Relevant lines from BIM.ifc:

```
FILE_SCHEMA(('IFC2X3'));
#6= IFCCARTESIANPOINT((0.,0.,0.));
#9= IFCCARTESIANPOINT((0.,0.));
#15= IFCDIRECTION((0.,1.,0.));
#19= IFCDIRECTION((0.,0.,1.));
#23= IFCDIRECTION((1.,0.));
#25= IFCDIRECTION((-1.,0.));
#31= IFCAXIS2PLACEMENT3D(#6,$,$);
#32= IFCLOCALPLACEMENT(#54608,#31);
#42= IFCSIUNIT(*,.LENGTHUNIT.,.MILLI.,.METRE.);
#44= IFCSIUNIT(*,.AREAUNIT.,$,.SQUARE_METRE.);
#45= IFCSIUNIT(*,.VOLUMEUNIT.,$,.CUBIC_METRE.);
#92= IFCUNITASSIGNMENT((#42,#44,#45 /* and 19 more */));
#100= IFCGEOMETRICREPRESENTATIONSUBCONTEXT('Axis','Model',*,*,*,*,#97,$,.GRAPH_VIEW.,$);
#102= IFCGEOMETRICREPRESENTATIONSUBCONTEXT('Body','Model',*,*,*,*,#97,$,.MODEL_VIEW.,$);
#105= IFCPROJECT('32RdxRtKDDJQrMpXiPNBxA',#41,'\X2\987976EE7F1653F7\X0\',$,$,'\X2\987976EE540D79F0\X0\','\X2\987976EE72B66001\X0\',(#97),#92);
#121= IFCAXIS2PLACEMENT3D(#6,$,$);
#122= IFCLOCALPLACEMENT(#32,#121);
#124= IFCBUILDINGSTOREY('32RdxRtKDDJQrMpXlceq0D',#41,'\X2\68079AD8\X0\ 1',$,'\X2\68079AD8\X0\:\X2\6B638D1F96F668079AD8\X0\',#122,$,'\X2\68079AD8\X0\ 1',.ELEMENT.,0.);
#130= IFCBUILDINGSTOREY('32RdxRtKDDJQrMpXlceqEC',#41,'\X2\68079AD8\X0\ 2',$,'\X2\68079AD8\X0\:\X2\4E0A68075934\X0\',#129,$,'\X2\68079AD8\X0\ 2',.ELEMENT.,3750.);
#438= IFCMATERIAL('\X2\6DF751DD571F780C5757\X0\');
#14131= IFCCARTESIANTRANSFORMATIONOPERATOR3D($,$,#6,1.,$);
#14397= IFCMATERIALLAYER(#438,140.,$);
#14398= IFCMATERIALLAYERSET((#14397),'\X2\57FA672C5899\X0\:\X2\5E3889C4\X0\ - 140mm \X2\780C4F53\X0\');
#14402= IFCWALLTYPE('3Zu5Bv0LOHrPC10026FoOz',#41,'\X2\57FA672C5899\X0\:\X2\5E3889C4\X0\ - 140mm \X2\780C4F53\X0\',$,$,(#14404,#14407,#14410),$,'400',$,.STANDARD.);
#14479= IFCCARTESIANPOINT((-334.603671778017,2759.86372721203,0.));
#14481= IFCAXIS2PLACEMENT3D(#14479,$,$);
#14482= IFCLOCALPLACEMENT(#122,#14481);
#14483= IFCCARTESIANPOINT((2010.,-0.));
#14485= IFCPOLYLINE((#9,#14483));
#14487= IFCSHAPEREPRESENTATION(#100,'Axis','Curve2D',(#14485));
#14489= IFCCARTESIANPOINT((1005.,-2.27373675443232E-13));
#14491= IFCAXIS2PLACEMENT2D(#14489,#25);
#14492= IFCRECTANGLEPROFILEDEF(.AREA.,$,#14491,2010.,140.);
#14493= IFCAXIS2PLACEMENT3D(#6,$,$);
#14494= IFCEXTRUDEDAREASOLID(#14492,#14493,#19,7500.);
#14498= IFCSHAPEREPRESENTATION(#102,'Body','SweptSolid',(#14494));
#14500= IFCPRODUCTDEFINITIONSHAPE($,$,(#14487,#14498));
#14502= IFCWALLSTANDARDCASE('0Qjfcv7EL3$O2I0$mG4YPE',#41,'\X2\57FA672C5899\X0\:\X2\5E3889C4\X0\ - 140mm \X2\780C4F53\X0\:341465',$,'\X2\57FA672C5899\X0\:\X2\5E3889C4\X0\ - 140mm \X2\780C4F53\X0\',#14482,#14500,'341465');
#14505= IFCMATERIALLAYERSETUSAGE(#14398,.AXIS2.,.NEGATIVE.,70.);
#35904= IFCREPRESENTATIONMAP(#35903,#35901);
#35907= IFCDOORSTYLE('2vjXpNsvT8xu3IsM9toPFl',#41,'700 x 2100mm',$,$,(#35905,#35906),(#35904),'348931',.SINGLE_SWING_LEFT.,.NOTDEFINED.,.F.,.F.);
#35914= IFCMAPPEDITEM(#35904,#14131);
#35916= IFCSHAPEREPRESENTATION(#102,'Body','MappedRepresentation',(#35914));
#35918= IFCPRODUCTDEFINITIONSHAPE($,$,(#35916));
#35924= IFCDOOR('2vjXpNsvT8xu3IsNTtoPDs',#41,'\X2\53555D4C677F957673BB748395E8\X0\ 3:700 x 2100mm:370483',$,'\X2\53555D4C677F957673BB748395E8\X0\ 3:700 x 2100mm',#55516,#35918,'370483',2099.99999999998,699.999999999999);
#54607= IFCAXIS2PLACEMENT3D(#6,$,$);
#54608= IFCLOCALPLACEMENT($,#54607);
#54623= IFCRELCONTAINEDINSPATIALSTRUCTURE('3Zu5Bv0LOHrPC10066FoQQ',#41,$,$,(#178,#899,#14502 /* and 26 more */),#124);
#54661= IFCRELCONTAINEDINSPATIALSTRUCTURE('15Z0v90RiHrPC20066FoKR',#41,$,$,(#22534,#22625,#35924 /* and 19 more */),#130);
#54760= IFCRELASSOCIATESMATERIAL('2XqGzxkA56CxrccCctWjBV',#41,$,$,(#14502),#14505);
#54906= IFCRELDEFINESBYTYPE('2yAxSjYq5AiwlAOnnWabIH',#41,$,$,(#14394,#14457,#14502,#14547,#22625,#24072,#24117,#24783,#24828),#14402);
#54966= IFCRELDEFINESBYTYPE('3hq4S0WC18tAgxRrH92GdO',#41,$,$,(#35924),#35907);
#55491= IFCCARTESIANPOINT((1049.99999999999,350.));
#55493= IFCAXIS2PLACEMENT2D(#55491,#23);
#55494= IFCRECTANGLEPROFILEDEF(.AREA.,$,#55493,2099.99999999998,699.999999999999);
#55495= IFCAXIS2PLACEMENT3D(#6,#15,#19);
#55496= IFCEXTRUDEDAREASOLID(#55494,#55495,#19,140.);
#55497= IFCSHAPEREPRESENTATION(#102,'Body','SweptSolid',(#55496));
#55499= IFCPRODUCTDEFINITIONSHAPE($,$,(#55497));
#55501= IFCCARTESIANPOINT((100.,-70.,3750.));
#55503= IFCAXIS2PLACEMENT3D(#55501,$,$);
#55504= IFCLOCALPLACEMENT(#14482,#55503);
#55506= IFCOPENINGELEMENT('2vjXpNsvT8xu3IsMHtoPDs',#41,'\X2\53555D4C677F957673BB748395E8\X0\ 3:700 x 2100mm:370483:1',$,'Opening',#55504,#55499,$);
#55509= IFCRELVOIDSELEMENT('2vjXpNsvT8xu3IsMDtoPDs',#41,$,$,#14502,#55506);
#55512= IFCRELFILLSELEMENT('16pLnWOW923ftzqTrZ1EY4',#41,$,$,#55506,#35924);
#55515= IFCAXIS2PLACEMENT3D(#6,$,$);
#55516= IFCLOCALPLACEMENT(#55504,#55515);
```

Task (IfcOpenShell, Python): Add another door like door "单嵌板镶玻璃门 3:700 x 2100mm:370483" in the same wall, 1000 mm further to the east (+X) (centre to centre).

```python
import ifcopenshell
import ifcopenshell.api.feature
import ifcopenshell.api.geometry
import ifcopenshell.api.root
import ifcopenshell.geom
import ifcopenshell.util.element
import ifcopenshell.util.placement
import ifcopenshell.util.shape

model = ifcopenshell.open("BIM.ifc")
settings = ifcopenshell.geom.settings()


def volume(element):
    """Net volume in cubic metres, openings subtracted."""
    shape = ifcopenshell.geom.create_shape(settings, element)
    return ifcopenshell.util.shape.get_volume(shape.geometry)


def reuse_history(source, copy):
    """copy_class also copies each property set's owner history, people and application; keep the originals."""
    for rel in copy.IsDefinedBy:
        if rel.is_a("IfcRelDefinesByProperties") and (history := rel.RelatingPropertyDefinition.OwnerHistory):
            rel.RelatingPropertyDefinition.OwnerHistory = source.OwnerHistory
            ifcopenshell.util.element.remove_deep2(model, history)


door = model.by_guid("2vjXpNsvT8xu3IsNTtoPDs")
opening = door.FillsVoids[0].RelatingOpeningElement
wall = opening.VoidsElements[0].RelatingBuildingElement
before = volume(wall)
shift = ifcopenshell.util.placement.get_local_placement(wall.ObjectPlacement)[:3, 0] * 1000.0

# copy_class copies the void relationship, type, container and properties, but no geometry.
new_opening = ifcopenshell.api.root.copy_class(model, product=opening)
new_opening.Representation = ifcopenshell.util.element.copy_deep(
    model, opening.Representation, exclude=["IfcGeometricRepresentationContext", "IfcRepresentationMap"]
)
new_opening.Name = "单嵌板镶玻璃门 3:700 x 2100mm"
new_door = ifcopenshell.api.root.copy_class(model, product=door)
new_door.Representation = ifcopenshell.util.element.copy_deep(
    model, door.Representation, exclude=["IfcGeometricRepresentationContext", "IfcRepresentationMap"]
)
new_door.Name = "单嵌板镶玻璃门 3:700 x 2100mm"
new_door.Tag = None
reuse_history(door, new_door)
fills = ifcopenshell.api.feature.add_filling(model, opening=new_opening, element=new_door)
fills.OwnerHistory = new_door.OwnerHistory  # required in IFC2X3

for old, new in ((opening, new_opening), (door, new_door)):
    matrix = ifcopenshell.util.placement.get_local_placement(old.ObjectPlacement)
    matrix[:3, 3] += shift
    ifcopenshell.api.geometry.edit_object_placement(model, product=new, matrix=matrix, is_si=False)

after = volume(wall)

print(f"wall volume {before:.3f} -> {after:.3f} m3")

model.write("BIM_updated.ifc")
```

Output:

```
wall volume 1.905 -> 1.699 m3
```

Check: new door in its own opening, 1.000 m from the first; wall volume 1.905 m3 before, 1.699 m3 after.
